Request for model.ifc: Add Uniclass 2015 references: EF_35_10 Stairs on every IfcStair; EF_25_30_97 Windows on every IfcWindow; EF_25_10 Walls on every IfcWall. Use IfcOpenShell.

First a look at what the model holds.

```python
import ifcopenshell

model = ifcopenshell.open("model.ifc")
print(model.schema)
print("classifications:", [c.Name for c in model.by_type("IfcClassification")])
for ifc_class in ("IfcDoor", "IfcRoof", "IfcStair", "IfcWall", "IfcWindow"):
    print(ifc_class, len(model.by_type(ifc_class)))
```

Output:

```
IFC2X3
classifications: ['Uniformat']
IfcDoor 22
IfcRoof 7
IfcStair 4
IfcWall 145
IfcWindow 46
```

```python
import ifcopenshell
import ifcopenshell.api.classification

model = ifcopenshell.open("model.ifc")

# IFC2X3 requires Source and Edition and has no link from the project to the system.
system = model.create_entity("IfcClassification", Source="NBS", Edition="2015", Name="Uniclass 2015")

codes = {
    "IfcStair": ("EF_35_10", "Stairs"),
    "IfcWindow": ("EF_25_30_97", "Windows"),
    "IfcWall": ("EF_25_10", "Walls"),
}
for ifc_class, (code, name) in codes.items():
    products = model.by_type(ifc_class)
    ifcopenshell.api.classification.add_reference(
        model, products=products, classification=system, identification=code, name=name
    )
    print(code, len(products))

model.write("model_updated.ifc")
```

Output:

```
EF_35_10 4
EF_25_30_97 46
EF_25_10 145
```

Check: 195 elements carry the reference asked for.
